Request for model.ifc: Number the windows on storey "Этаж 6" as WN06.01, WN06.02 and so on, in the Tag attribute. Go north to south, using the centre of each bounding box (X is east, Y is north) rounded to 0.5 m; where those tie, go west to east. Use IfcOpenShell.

First a look at what the model holds.

```python
import ifcopenshell
import ifcopenshell.util.element
import ifcopenshell.util.placement

model = ifcopenshell.open("model.ifc")
print(model.schema)
storey = next(s for s in model.by_type("IfcBuildingStorey") if s.Name == "Этаж 6")
windows = [e for e in ifcopenshell.util.element.get_decomposition(storey) if e.is_a("IfcWindow")]
for e in sorted(windows, key=lambda e: e.id()):
    origin = ifcopenshell.util.placement.get_local_placement(e.ObjectPlacement)[:3, 3]
    print(e.id(), e.Tag, e.Name, origin.round(2) + 0.0, sep=" | ")
```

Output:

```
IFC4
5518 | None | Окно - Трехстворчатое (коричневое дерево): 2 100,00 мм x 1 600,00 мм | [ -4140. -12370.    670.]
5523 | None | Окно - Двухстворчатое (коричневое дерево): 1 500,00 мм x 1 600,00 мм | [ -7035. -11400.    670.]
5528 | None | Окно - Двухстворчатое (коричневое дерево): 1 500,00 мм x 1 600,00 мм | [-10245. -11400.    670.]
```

```python
import ifcopenshell
import ifcopenshell.geom
import ifcopenshell.util.element
import ifcopenshell.util.shape

model = ifcopenshell.open("model.ifc")
settings = ifcopenshell.geom.settings()
settings.set("use-world-coords", True)


def centre(element):
    shape = ifcopenshell.geom.create_shape(settings, element)
    return ifcopenshell.util.shape.get_bbox_centroid(shape.geometry)


storey = next(s for s in model.by_type("IfcBuildingStorey") if s.Name == "Этаж 6")
windows = [e for e in ifcopenshell.util.element.get_decomposition(storey) if e.is_a("IfcWindow")]

# Insertion points can sit at a corner or the storey origin, so sort by the geometry (in metres).
centres = {e: centre(e) for e in windows}
windows.sort(key=lambda e: (-round(centres[e][1] / 0.5), centres[e][0]))

for i, e in enumerate(windows, start=1):
    number = f"WN06.{i:02d}"
    e.Tag = number
    print(e.id(), number)

model.write("model-out.ifc")
```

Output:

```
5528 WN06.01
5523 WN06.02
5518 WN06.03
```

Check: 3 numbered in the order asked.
